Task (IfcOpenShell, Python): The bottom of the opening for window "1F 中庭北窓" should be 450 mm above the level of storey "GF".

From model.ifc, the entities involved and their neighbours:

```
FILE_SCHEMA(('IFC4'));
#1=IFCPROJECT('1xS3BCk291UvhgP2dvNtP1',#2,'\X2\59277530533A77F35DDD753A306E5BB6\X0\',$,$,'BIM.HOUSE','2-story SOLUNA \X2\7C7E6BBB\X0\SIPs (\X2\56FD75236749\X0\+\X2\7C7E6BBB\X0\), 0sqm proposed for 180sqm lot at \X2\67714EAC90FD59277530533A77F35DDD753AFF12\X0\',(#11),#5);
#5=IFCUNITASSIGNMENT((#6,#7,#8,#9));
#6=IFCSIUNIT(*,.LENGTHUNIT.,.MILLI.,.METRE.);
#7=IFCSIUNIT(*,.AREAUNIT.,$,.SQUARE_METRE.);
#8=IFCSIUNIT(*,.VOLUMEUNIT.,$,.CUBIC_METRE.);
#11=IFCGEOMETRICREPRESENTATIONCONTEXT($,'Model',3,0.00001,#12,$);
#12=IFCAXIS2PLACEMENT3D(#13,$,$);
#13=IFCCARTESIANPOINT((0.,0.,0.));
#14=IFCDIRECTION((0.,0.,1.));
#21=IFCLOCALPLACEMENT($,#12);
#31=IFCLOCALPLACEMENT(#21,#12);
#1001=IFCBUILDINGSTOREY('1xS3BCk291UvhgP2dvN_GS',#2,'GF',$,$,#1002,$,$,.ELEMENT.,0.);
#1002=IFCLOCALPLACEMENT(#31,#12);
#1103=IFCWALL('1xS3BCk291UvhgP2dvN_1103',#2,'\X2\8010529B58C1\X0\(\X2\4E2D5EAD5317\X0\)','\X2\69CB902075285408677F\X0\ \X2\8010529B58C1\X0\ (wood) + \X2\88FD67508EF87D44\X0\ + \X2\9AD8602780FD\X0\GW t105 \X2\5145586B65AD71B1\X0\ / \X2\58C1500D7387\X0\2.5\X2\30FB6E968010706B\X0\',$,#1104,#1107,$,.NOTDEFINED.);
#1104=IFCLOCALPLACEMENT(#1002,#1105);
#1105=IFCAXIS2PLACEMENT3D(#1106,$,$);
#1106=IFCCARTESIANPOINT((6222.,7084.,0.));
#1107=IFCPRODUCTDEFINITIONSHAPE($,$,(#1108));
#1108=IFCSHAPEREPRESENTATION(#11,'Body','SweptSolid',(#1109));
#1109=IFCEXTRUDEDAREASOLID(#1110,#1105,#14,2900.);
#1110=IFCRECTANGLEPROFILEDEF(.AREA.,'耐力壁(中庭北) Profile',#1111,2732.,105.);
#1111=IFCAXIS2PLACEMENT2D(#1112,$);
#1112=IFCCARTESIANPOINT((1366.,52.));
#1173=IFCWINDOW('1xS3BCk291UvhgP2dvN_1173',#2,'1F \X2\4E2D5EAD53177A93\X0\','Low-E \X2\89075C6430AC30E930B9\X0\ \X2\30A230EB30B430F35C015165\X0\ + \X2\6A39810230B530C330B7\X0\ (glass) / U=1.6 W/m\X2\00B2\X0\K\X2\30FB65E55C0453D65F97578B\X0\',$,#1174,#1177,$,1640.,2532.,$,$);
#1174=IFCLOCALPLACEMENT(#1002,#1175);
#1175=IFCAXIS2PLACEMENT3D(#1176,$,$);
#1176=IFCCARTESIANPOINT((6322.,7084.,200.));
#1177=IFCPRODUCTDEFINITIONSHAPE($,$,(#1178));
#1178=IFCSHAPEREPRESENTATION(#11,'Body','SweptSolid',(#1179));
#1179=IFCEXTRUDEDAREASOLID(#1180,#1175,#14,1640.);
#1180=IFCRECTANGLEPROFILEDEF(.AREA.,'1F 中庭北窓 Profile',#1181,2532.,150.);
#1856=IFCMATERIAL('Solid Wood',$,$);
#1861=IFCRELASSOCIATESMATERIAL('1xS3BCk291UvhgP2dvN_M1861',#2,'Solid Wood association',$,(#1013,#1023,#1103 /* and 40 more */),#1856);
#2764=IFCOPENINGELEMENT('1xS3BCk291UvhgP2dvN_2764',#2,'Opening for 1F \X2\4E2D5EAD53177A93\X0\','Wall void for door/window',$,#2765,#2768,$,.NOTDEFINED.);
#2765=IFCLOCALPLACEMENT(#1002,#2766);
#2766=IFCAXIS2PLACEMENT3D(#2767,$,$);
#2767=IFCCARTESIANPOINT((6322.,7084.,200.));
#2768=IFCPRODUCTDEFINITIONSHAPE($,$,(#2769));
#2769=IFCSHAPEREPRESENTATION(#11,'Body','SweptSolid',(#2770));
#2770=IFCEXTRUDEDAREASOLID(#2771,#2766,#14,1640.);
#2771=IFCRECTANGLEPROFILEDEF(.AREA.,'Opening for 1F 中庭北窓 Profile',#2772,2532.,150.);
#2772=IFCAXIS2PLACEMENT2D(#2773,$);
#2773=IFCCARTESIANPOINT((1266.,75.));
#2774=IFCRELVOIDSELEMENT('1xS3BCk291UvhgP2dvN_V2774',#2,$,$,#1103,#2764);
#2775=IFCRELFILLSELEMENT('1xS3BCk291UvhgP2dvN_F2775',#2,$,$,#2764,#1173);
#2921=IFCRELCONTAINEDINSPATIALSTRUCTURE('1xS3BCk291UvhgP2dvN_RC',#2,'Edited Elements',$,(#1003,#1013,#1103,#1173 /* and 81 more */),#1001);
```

```python
import numpy as np
import ifcopenshell
import ifcopenshell.api.geometry
import ifcopenshell.geom
import ifcopenshell.util.element
import ifcopenshell.util.placement
import ifcopenshell.util.shape
import ifcopenshell.util.unit

model = ifcopenshell.open("model.ifc")
unit_scale = ifcopenshell.util.unit.calculate_unit_scale(model)

window = model.by_guid("1xS3BCk291UvhgP2dvN_1173")
opening = window.FillsVoids[0].RelatingOpeningElement
storey = ifcopenshell.util.element.get_container(window, ifc_class="IfcBuildingStorey")
level = ifcopenshell.util.placement.get_local_placement(storey.ObjectPlacement)[2, 3]

# The opening's origin need not be at the sill, so measure its lowest point.
shape = ifcopenshell.geom.create_shape(ifcopenshell.geom.settings(), opening)
bottom = ifcopenshell.util.shape.get_shape_bottom_elevation(shape, shape.geometry) / unit_scale
dz = level + 0.45 / unit_scale - bottom

shift = np.array([0.0, 0.0, dz])
# The window is not placed relative to its opening, so move both.
for product in (opening, window):
    matrix = ifcopenshell.util.placement.get_local_placement(product.ObjectPlacement)
    matrix[:3, 3] += shift
    ifcopenshell.api.geometry.edit_object_placement(model, product=product, matrix=matrix, is_si=False)

print(f"moved by {dz * unit_scale:+.3f} m")

model.write("model_rev.ifc")
```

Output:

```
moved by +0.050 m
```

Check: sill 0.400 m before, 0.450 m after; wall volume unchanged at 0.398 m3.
